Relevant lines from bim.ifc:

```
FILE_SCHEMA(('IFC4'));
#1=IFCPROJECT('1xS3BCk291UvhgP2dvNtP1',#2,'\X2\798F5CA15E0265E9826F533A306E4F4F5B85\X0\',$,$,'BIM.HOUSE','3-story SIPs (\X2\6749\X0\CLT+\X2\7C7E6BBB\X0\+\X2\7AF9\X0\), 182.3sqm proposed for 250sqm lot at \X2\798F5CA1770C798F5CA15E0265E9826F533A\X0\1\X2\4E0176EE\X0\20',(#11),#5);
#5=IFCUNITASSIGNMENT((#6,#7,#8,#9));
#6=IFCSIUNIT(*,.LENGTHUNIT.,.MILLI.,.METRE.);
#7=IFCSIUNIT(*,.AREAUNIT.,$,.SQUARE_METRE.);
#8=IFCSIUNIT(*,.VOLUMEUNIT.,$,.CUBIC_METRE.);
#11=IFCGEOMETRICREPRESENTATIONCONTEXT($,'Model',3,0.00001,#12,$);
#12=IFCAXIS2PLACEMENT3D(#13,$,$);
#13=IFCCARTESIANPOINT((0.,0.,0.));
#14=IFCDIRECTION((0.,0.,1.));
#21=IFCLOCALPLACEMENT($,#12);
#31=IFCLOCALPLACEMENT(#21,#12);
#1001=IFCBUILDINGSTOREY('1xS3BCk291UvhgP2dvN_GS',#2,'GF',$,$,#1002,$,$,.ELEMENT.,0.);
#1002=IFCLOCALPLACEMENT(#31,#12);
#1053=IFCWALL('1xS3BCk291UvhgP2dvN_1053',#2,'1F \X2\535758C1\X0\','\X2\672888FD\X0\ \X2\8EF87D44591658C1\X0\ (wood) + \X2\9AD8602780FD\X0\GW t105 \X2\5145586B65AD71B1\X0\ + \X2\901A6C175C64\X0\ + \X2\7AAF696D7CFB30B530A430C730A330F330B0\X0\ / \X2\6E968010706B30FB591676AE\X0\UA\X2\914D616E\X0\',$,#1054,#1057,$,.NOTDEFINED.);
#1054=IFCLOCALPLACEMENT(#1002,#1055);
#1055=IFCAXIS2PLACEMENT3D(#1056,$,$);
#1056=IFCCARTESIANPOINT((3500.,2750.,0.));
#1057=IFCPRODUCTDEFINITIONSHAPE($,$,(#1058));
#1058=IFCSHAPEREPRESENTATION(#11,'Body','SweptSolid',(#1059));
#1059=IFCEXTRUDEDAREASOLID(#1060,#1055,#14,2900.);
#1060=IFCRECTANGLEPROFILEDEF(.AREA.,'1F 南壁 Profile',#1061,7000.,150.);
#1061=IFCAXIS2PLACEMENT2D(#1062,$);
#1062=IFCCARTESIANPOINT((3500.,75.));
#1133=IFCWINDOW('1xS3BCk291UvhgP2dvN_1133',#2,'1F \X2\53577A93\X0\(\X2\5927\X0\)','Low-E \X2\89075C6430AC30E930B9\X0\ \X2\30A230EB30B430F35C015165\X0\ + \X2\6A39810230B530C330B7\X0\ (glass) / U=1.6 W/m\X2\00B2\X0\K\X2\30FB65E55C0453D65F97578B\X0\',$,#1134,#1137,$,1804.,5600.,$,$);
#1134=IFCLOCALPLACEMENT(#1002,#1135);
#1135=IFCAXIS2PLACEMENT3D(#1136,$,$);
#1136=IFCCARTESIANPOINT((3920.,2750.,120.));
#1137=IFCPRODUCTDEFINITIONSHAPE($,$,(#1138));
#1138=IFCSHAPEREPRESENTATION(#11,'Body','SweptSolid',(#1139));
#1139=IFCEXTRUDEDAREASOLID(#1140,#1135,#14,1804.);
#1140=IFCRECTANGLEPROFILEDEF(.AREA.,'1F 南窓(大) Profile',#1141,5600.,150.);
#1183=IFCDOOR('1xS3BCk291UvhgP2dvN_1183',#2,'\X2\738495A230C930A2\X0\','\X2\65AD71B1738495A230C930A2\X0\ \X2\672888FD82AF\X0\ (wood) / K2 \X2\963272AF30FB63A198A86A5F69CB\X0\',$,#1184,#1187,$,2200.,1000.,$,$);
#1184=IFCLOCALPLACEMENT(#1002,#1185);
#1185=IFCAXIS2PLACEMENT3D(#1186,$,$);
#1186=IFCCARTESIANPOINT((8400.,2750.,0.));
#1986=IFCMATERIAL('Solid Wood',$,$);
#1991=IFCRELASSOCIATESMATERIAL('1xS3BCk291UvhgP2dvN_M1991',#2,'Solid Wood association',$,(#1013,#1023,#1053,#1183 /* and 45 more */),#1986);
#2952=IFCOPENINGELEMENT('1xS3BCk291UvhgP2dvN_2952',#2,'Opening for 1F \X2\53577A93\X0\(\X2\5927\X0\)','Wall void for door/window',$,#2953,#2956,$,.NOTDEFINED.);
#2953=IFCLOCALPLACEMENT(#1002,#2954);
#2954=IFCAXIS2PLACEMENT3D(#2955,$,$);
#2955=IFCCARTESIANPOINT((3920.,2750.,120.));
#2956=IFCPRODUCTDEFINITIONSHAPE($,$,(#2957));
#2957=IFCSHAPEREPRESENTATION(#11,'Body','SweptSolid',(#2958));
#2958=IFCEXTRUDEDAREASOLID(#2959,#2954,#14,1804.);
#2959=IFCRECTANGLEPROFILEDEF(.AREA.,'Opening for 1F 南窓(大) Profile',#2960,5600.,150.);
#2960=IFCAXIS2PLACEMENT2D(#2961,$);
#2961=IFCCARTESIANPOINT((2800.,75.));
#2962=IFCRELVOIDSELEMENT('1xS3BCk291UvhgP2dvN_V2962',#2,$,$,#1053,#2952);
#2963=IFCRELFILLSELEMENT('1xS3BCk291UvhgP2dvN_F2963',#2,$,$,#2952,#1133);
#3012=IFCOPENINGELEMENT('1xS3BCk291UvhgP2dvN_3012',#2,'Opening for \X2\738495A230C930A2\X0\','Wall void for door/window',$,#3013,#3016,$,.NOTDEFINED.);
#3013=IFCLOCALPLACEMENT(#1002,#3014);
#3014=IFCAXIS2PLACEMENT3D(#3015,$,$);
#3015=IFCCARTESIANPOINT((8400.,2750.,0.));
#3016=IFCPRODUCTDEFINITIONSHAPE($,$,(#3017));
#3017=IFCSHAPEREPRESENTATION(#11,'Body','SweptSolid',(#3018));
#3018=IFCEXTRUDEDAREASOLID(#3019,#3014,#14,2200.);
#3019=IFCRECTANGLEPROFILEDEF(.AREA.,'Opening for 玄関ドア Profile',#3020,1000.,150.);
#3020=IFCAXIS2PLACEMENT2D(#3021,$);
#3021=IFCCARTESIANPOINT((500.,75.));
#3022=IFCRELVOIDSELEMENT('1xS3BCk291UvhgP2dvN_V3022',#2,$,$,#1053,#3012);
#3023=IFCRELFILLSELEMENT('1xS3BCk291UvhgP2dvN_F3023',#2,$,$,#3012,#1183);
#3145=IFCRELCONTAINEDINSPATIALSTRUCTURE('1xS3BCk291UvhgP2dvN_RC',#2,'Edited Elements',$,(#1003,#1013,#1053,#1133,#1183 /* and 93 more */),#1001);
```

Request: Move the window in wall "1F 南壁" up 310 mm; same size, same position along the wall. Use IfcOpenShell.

```python
import numpy as np
import ifcopenshell
import ifcopenshell.api.geometry
import ifcopenshell.util.placement
import ifcopenshell.util.unit

model = ifcopenshell.open("bim.ifc")
unit_scale = ifcopenshell.util.unit.calculate_unit_scale(model)

window = model.by_guid("1xS3BCk291UvhgP2dvN_1133")
opening = window.FillsVoids[0].RelatingOpeningElement
dz = 0.31 / unit_scale

shift = np.array([0.0, 0.0, dz])
# The window is not placed relative to its opening, so move both.
for product in (opening, window):
    matrix = ifcopenshell.util.placement.get_local_placement(product.ObjectPlacement)
    matrix[:3, 3] += shift
    ifcopenshell.api.geometry.edit_object_placement(model, product=product, matrix=matrix, is_si=False)

print(f"moved by {dz * unit_scale:+.3f} m")

model.write("bim_updated.ifc")
```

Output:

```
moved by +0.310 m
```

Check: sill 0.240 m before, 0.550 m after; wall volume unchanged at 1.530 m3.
